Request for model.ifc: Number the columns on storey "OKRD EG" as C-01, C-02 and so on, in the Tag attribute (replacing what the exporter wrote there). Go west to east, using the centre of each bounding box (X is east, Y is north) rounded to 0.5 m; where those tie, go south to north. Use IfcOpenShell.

First a look at what the model holds.

```python
import ifcopenshell
import ifcopenshell.util.element
import ifcopenshell.util.placement

model = ifcopenshell.open("model.ifc")
print(model.schema)
storey = next(s for s in model.by_type("IfcBuildingStorey") if s.Name == "OKRD EG")
columns = [e for e in ifcopenshell.util.element.get_decomposition(storey) if e.is_a("IfcColumn")]
for e in sorted(columns, key=lambda e: e.id()):
    origin = ifcopenshell.util.placement.get_local_placement(e.ObjectPlacement)[:3, 3]
    print(e.id(), e.Tag, e.Name, origin.round(2) + 0.0, sep=" | ")
```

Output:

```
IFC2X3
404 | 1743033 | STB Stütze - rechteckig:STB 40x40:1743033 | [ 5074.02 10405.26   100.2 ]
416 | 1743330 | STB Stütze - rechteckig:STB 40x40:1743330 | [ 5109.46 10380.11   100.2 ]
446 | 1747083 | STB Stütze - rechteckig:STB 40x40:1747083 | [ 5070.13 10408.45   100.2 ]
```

```python
import ifcopenshell
import ifcopenshell.geom
import ifcopenshell.util.element
import ifcopenshell.util.shape

model = ifcopenshell.open("model.ifc")
settings = ifcopenshell.geom.settings()
settings.set("use-world-coords", True)


def centre(element):
    shape = ifcopenshell.geom.create_shape(settings, element)
    return ifcopenshell.util.shape.get_bbox_centroid(shape.geometry)


storey = next(s for s in model.by_type("IfcBuildingStorey") if s.Name == "OKRD EG")
columns = [e for e in ifcopenshell.util.element.get_decomposition(storey) if e.is_a("IfcColumn")]

# Insertion points can sit at a corner or the storey origin, so sort by the geometry (in metres).
centres = {e: centre(e) for e in columns}
columns.sort(key=lambda e: (round(centres[e][0] / 0.5), centres[e][1]))

for i, e in enumerate(columns, start=1):
    number = f"C-{i:02d}"
    e.Tag = number
    print(e.id(), number)

model.write("model_updated.ifc")
```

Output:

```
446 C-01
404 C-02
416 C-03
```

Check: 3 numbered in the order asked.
